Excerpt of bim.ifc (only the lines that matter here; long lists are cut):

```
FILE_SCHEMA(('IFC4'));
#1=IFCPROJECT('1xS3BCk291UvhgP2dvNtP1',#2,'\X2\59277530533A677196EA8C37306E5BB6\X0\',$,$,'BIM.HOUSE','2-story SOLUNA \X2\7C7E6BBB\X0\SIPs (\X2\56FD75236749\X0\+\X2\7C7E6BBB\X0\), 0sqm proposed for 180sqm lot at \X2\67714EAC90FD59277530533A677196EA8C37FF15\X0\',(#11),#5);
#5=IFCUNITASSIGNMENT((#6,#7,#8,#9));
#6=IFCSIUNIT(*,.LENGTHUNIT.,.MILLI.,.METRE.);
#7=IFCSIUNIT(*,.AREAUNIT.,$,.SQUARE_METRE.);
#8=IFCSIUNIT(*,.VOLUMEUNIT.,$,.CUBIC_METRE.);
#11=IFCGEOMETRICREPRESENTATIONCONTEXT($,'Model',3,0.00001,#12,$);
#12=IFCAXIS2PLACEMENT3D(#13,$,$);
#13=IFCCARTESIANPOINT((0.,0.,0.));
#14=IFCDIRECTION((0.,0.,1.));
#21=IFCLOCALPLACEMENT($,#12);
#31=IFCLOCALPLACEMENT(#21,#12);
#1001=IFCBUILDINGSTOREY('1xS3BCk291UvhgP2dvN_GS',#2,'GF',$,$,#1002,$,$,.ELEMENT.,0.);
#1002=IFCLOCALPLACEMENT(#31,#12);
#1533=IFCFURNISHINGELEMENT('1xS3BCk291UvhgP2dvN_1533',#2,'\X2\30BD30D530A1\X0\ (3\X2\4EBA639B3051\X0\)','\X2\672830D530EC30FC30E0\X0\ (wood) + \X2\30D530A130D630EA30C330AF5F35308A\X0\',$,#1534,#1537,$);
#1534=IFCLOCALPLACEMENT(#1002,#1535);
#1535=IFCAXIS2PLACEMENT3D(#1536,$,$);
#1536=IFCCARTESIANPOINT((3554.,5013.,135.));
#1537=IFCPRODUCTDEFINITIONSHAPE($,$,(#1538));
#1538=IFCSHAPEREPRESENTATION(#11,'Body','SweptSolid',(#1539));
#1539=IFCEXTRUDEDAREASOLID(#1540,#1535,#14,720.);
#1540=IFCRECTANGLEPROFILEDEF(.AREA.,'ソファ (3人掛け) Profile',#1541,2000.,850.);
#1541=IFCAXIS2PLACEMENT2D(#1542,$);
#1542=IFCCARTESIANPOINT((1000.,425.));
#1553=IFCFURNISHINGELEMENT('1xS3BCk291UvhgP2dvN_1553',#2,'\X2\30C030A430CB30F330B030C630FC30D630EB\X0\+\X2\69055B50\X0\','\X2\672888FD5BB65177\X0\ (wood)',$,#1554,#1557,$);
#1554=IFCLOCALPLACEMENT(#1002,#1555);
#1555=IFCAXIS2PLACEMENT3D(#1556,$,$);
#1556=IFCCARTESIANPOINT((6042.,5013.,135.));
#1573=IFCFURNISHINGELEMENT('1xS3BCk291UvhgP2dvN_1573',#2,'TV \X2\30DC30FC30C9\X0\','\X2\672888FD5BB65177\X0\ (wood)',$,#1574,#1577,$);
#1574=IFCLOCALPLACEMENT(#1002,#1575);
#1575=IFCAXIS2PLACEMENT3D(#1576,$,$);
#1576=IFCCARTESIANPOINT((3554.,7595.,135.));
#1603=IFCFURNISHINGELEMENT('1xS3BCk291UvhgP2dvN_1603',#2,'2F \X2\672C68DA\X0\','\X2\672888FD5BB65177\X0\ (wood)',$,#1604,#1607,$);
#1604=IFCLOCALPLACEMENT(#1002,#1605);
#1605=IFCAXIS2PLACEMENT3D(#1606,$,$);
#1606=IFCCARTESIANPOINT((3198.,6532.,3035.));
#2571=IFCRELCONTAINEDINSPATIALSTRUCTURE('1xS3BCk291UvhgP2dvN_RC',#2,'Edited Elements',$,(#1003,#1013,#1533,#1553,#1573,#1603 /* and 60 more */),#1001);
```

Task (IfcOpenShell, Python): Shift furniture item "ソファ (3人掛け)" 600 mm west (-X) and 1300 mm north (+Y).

```python
import ifcopenshell
import ifcopenshell.api.geometry
import ifcopenshell.util.placement
import ifcopenshell.util.unit

model = ifcopenshell.open("bim.ifc")
unit_scale = ifcopenshell.util.unit.calculate_unit_scale(model)

item = model.by_guid("1xS3BCk291UvhgP2dvN_1533")
matrix = ifcopenshell.util.placement.get_local_placement(item.ObjectPlacement)
matrix[0, 3] -= 0.6 / unit_scale
matrix[1, 3] += 1.3 / unit_scale
ifcopenshell.api.geometry.edit_object_placement(model, product=item, matrix=matrix, is_si=False)

print(ifcopenshell.util.placement.get_local_placement(item.ObjectPlacement).round(3) + 0.0)

model.write("bim_rev.ifc")
```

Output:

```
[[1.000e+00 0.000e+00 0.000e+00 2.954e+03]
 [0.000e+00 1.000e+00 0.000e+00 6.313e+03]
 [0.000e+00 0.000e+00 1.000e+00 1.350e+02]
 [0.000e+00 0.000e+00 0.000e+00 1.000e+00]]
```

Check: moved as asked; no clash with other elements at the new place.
